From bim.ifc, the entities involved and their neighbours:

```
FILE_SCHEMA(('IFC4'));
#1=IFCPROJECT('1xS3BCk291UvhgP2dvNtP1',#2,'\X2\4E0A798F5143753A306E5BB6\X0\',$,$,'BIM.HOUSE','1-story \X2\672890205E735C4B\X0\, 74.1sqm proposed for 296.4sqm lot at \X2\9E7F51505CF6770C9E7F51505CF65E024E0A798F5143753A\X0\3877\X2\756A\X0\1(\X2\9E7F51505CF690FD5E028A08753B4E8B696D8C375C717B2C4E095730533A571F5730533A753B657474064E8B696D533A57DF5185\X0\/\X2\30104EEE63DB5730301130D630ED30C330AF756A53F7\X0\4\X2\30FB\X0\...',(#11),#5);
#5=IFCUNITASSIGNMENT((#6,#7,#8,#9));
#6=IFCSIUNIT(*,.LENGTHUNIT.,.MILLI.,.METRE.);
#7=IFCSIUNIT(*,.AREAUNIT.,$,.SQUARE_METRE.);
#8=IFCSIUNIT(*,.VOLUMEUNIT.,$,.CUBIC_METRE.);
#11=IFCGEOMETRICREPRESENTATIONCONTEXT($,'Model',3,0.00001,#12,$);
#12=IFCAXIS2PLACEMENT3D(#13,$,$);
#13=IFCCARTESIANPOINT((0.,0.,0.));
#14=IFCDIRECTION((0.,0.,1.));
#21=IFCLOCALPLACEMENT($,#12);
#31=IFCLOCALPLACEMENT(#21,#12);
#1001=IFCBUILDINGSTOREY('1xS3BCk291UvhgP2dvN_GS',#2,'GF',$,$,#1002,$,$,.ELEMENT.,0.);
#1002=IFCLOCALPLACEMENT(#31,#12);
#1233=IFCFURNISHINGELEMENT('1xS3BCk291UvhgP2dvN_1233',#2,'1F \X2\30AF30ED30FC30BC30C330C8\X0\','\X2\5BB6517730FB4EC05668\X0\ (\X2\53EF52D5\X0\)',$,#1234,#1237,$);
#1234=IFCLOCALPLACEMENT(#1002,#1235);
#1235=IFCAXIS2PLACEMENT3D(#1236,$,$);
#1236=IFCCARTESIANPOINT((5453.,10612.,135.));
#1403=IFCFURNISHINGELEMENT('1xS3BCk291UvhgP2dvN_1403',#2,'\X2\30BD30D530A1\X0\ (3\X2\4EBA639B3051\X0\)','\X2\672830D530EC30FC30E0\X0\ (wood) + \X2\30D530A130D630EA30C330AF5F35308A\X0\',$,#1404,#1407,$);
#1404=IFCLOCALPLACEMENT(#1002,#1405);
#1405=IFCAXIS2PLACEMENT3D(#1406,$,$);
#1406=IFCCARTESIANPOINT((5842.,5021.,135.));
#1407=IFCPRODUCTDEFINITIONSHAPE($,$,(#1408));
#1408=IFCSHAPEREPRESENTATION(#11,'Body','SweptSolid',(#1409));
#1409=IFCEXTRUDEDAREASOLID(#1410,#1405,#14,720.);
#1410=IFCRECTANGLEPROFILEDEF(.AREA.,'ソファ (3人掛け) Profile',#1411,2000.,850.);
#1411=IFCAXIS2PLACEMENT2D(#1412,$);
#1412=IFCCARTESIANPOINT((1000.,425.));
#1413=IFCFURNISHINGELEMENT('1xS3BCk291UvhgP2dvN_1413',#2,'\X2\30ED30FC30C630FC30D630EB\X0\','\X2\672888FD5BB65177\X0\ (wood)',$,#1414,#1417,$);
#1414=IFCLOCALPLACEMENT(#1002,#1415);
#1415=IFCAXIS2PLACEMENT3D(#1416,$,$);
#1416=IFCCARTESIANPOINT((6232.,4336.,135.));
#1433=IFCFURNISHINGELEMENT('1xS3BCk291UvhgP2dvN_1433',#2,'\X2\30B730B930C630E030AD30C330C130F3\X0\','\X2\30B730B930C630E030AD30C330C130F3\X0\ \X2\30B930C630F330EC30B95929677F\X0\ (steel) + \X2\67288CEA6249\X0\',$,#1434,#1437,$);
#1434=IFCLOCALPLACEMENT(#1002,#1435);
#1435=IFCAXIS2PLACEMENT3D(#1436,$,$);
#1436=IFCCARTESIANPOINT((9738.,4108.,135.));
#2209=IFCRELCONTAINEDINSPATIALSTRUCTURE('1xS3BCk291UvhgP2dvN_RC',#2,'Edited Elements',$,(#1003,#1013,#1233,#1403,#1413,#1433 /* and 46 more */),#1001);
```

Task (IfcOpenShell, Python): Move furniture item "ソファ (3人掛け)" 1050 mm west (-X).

```python
import ifcopenshell
import ifcopenshell.api.geometry
import ifcopenshell.util.placement
import ifcopenshell.util.unit

model = ifcopenshell.open("bim.ifc")
unit_scale = ifcopenshell.util.unit.calculate_unit_scale(model)

item = model.by_guid("1xS3BCk291UvhgP2dvN_1403")
matrix = ifcopenshell.util.placement.get_local_placement(item.ObjectPlacement)
matrix[0, 3] -= 1.05 / unit_scale
ifcopenshell.api.geometry.edit_object_placement(model, product=item, matrix=matrix, is_si=False)

print(ifcopenshell.util.placement.get_local_placement(item.ObjectPlacement).round(3) + 0.0)

model.write("bim_updated.ifc")
```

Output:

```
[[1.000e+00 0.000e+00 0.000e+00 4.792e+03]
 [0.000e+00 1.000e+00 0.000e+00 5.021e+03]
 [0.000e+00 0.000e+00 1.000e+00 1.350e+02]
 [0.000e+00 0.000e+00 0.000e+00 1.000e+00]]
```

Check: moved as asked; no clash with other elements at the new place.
